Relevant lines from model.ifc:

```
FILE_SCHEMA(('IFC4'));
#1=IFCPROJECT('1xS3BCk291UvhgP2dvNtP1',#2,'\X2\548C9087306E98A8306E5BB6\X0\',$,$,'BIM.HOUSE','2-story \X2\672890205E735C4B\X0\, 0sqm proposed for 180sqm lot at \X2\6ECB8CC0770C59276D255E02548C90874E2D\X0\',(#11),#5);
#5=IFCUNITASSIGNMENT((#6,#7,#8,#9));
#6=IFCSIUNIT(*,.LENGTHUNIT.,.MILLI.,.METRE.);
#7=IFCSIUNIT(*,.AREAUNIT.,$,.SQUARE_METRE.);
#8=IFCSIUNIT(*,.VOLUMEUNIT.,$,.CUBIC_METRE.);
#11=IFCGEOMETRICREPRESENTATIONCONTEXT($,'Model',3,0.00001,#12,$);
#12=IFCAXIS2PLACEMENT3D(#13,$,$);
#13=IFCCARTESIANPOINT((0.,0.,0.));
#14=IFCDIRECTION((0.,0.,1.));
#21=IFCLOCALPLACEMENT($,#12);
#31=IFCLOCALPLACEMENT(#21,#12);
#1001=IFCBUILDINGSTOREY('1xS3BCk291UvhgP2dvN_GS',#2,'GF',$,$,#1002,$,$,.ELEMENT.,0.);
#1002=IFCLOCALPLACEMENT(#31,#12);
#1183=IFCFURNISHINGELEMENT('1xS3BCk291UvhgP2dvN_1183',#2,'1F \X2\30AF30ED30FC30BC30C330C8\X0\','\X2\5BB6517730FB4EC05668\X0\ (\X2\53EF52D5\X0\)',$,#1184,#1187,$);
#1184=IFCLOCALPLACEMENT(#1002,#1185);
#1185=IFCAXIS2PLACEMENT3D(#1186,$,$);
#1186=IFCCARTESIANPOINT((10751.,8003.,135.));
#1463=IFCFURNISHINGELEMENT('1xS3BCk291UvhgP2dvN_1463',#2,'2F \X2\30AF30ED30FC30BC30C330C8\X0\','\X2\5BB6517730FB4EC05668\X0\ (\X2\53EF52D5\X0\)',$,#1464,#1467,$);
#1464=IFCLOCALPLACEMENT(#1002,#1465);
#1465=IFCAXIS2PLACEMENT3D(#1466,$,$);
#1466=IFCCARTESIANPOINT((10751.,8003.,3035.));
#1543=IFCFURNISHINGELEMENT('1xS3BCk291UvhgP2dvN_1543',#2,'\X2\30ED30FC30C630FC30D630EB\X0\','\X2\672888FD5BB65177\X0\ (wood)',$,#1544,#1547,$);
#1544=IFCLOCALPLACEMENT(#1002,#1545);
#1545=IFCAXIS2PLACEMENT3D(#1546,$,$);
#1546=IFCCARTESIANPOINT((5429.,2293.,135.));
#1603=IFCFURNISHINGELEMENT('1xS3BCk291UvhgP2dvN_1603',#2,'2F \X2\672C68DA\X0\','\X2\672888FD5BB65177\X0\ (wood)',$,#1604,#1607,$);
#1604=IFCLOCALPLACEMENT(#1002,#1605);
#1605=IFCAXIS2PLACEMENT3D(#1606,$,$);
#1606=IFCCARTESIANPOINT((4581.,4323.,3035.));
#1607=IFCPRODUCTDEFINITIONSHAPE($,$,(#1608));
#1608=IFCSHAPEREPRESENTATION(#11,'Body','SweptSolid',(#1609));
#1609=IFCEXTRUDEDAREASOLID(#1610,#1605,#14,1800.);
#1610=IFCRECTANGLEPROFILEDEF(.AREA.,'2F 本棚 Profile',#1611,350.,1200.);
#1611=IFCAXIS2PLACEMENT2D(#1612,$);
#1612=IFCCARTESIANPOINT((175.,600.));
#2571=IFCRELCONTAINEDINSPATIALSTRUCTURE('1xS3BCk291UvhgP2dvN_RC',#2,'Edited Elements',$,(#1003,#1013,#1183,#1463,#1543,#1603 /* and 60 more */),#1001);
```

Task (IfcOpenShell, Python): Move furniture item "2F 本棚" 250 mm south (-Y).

```python
import ifcopenshell
import ifcopenshell.api.geometry
import ifcopenshell.util.placement

model = ifcopenshell.open("model.ifc")

item = model.by_id(1603)
matrix = ifcopenshell.util.placement.get_local_placement(item.ObjectPlacement)
matrix[1, 3] -= 250.0
ifcopenshell.api.geometry.edit_object_placement(model, product=item, matrix=matrix, is_si=False)

print(ifcopenshell.util.placement.get_local_placement(item.ObjectPlacement).round(3) + 0.0)

model.write("model_rev.ifc")
```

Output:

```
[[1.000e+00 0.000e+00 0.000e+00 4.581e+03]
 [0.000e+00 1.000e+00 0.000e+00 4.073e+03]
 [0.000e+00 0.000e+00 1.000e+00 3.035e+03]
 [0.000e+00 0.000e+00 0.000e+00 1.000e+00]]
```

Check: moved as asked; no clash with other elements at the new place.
